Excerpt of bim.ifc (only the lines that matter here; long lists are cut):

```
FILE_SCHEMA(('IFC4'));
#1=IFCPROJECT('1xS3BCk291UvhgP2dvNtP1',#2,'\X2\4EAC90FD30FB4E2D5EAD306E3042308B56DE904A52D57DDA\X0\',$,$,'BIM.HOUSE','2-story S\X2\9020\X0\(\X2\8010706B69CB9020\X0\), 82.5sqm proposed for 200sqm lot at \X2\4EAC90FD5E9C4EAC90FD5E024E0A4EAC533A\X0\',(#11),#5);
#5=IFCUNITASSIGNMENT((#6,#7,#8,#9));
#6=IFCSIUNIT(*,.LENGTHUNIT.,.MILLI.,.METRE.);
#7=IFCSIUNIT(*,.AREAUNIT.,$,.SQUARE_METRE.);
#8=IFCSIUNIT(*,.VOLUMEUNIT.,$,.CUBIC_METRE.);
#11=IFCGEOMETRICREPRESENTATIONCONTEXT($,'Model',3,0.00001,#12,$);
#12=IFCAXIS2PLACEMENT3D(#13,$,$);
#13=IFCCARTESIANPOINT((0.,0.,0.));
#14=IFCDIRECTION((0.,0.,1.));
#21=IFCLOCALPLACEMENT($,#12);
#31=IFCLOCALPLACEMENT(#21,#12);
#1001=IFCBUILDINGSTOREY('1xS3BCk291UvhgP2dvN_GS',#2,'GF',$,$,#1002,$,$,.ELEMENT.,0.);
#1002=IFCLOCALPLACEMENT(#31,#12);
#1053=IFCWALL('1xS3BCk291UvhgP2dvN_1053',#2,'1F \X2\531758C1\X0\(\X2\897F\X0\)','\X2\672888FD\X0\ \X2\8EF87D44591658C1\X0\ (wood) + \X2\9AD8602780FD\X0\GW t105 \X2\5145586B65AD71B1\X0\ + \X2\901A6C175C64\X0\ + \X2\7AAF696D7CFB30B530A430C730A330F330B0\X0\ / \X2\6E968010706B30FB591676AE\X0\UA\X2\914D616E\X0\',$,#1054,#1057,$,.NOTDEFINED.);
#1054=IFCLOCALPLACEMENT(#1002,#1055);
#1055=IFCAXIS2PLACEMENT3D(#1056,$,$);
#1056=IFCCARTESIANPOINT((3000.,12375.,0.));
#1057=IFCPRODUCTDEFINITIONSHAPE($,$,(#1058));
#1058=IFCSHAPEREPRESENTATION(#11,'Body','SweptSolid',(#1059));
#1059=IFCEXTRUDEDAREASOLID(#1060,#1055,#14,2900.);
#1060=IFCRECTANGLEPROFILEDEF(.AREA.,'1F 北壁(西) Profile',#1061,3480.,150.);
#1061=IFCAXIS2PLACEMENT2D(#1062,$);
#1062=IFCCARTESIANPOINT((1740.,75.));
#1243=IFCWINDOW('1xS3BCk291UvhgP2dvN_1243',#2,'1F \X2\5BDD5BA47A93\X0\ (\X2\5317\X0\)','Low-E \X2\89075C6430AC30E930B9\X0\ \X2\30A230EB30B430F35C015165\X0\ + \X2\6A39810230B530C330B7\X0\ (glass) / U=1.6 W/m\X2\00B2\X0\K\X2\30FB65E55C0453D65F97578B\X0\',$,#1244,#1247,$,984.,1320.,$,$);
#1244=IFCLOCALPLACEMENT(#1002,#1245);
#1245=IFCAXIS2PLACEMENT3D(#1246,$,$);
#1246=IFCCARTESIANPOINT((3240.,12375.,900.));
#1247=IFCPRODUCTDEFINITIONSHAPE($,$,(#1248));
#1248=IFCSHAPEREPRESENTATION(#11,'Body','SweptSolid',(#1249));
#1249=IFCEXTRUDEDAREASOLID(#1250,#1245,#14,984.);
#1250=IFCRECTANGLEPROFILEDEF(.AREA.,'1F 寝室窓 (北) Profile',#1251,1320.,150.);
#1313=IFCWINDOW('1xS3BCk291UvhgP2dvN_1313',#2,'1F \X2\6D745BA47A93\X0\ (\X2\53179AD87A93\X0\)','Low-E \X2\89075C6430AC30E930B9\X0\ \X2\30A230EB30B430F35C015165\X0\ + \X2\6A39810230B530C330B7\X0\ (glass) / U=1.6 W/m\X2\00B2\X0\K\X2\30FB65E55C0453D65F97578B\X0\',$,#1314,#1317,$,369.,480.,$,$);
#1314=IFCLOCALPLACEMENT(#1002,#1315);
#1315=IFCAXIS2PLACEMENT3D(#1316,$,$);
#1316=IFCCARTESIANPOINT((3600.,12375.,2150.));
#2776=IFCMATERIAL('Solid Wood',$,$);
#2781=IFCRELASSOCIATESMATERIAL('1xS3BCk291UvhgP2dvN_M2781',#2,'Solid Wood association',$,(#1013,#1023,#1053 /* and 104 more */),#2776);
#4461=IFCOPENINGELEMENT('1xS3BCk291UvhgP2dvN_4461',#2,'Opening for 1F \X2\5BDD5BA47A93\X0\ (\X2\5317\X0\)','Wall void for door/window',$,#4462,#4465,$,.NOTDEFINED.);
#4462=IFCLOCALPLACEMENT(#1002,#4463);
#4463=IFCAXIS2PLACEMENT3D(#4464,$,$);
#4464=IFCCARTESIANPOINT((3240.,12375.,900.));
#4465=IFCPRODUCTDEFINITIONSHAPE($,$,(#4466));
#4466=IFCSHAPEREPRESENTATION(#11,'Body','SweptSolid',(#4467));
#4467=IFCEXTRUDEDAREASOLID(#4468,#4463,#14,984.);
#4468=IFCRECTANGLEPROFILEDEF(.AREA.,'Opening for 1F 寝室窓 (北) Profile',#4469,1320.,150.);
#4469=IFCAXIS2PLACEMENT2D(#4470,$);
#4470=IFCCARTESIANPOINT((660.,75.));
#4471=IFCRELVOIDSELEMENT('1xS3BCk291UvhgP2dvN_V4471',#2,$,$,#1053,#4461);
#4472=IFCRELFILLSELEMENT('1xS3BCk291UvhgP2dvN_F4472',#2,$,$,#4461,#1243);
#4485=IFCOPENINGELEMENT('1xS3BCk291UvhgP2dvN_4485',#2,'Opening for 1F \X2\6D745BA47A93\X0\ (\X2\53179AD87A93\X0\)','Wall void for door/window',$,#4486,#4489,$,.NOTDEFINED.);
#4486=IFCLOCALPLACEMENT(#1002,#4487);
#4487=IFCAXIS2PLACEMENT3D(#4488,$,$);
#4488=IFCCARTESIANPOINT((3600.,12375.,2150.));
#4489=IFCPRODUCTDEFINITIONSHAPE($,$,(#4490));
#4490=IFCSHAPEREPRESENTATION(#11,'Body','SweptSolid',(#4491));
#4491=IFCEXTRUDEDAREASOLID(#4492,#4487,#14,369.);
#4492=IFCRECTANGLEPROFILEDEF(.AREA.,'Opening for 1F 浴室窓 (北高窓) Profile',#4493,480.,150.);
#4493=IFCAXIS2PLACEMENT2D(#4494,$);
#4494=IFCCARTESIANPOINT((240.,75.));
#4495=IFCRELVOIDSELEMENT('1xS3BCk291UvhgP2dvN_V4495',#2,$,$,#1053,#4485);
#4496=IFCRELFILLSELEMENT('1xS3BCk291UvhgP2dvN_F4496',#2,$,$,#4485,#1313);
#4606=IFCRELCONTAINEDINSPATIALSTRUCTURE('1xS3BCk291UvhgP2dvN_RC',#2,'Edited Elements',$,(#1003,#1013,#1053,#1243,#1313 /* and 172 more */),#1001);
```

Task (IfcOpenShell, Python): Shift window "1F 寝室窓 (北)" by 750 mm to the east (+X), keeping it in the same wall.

```python
import ifcopenshell
import ifcopenshell.api.geometry
import ifcopenshell.util.placement
import ifcopenshell.util.unit

model = ifcopenshell.open("bim.ifc")
unit_scale = ifcopenshell.util.unit.calculate_unit_scale(model)

window = model.by_guid("1xS3BCk291UvhgP2dvN_1243")
opening = window.FillsVoids[0].RelatingOpeningElement
wall = opening.VoidsElements[0].RelatingBuildingElement

wall_matrix = ifcopenshell.util.placement.get_local_placement(wall.ObjectPlacement)
shift = wall_matrix[:3, 0] * 0.75 / unit_scale
before = ifcopenshell.util.placement.get_local_placement(window.ObjectPlacement)[:3, 3].copy()

# The window is not placed relative to its opening, so move both.
for product in (opening, window):
    matrix = ifcopenshell.util.placement.get_local_placement(product.ObjectPlacement)
    matrix[:3, 3] += shift
    ifcopenshell.api.geometry.edit_object_placement(model, product=product, matrix=matrix, is_si=False)

after = ifcopenshell.util.placement.get_local_placement(window.ObjectPlacement)[:3, 3]
print("window moved by", (after - before).round(3) + 0.0)

model.write("bim_edited.ifc")
```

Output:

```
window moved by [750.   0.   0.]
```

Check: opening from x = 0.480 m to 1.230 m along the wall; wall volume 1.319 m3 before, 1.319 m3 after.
